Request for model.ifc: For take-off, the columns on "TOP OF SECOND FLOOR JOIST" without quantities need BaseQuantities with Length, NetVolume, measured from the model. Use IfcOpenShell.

First a look at what the model holds.

```python
import ifcopenshell
import ifcopenshell.util.element
import ifcopenshell.util.unit

model = ifcopenshell.open("model.ifc")
print(model.schema)
for unit_type in ("LENGTHUNIT", "AREAUNIT", "VOLUMEUNIT"):
    print(unit_type, ifcopenshell.util.unit.calculate_unit_scale(model, unit_type))
storey = next(s for s in model.by_type("IfcBuildingStorey") if s.Name == "TOP OF SECOND FLOOR JOIST")
columns = [e for e in ifcopenshell.util.element.get_decomposition(storey) if e.is_a("IfcColumn")]
for e in sorted(columns, key=lambda e: e.id()):
    print(e.id(), e.is_a(), e.Name, list(ifcopenshell.util.element.get_psets(e, qtos_only=True)), sep=" | ")
```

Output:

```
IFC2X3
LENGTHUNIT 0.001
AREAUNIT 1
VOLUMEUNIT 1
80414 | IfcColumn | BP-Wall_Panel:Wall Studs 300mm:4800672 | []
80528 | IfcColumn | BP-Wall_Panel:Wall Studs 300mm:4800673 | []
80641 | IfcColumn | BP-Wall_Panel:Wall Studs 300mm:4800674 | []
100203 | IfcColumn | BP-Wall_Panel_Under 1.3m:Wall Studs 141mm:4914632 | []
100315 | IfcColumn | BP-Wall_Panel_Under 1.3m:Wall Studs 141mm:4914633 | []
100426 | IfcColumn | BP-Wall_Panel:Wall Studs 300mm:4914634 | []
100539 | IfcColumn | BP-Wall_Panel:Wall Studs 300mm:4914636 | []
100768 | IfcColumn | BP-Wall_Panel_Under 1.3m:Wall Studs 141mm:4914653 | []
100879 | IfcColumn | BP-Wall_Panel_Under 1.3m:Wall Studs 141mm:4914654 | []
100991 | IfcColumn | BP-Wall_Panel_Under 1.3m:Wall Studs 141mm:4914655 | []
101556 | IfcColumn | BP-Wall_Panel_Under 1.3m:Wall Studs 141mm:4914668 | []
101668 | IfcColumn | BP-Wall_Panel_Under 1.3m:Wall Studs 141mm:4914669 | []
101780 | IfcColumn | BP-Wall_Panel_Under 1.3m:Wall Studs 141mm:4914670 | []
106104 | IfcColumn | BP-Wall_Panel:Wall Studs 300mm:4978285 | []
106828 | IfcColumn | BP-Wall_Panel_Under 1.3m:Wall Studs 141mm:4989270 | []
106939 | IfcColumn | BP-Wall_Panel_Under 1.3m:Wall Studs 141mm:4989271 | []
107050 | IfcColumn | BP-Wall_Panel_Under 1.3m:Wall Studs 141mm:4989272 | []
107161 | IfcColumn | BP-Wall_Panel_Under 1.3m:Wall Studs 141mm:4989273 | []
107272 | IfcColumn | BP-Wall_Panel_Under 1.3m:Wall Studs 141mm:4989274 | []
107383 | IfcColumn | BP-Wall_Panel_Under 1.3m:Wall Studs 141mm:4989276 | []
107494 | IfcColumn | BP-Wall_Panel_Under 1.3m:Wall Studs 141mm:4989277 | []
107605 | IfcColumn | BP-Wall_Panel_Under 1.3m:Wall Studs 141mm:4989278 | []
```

```python
import ifcopenshell
import ifcopenshell.api.pset
import ifcopenshell.geom
import ifcopenshell.util.element
import ifcopenshell.util.shape
import ifcopenshell.util.unit

model = ifcopenshell.open("model.ifc")
unit_scale = ifcopenshell.util.unit.calculate_unit_scale(model)
volume_scale = ifcopenshell.util.unit.calculate_unit_scale(model, "VOLUMEUNIT")
settings = ifcopenshell.geom.settings()

storey = next(s for s in model.by_type("IfcBuildingStorey") if s.Name == "TOP OF SECOND FLOOR JOIST")
columns = [e for e in ifcopenshell.util.element.get_decomposition(storey) if e.is_a("IfcColumn")]

for e in sorted(columns, key=lambda e: e.id()):
    if ifcopenshell.util.element.get_psets(e, qtos_only=True, should_inherit=False):
        continue
    # Geometry comes back in metres, in the element's own axes.
    shape = ifcopenshell.geom.create_shape(settings, e)
    values = {
        "Length": ifcopenshell.util.shape.get_z(shape.geometry) / unit_scale,
        "NetVolume": ifcopenshell.util.shape.get_volume(shape.geometry) / volume_scale,
    }
    qto = ifcopenshell.api.pset.add_qto(model, product=e, name="BaseQuantities")
    ifcopenshell.api.pset.edit_qto(model, qto=qto, properties=values)
    print(e.id(), {k: round(v, 3) for k, v in values.items()})

model.write("model_edited.ifc")
```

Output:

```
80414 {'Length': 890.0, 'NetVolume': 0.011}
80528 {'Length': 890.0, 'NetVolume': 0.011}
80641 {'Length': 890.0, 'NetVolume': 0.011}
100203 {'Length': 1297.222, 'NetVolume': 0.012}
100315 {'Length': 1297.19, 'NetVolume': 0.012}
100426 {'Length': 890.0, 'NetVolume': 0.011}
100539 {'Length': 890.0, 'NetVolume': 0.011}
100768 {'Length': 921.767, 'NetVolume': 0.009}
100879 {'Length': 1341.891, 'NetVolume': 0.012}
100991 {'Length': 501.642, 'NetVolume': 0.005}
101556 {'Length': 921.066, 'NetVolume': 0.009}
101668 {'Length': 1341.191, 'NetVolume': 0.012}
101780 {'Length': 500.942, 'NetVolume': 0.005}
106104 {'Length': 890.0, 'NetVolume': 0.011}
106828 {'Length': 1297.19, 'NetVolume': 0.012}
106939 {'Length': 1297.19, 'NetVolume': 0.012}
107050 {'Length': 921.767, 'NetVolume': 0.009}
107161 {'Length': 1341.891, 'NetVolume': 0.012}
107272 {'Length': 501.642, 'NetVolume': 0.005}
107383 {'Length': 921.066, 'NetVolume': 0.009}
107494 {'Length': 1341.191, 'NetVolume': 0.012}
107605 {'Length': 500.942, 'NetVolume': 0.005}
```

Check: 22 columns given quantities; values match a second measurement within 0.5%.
